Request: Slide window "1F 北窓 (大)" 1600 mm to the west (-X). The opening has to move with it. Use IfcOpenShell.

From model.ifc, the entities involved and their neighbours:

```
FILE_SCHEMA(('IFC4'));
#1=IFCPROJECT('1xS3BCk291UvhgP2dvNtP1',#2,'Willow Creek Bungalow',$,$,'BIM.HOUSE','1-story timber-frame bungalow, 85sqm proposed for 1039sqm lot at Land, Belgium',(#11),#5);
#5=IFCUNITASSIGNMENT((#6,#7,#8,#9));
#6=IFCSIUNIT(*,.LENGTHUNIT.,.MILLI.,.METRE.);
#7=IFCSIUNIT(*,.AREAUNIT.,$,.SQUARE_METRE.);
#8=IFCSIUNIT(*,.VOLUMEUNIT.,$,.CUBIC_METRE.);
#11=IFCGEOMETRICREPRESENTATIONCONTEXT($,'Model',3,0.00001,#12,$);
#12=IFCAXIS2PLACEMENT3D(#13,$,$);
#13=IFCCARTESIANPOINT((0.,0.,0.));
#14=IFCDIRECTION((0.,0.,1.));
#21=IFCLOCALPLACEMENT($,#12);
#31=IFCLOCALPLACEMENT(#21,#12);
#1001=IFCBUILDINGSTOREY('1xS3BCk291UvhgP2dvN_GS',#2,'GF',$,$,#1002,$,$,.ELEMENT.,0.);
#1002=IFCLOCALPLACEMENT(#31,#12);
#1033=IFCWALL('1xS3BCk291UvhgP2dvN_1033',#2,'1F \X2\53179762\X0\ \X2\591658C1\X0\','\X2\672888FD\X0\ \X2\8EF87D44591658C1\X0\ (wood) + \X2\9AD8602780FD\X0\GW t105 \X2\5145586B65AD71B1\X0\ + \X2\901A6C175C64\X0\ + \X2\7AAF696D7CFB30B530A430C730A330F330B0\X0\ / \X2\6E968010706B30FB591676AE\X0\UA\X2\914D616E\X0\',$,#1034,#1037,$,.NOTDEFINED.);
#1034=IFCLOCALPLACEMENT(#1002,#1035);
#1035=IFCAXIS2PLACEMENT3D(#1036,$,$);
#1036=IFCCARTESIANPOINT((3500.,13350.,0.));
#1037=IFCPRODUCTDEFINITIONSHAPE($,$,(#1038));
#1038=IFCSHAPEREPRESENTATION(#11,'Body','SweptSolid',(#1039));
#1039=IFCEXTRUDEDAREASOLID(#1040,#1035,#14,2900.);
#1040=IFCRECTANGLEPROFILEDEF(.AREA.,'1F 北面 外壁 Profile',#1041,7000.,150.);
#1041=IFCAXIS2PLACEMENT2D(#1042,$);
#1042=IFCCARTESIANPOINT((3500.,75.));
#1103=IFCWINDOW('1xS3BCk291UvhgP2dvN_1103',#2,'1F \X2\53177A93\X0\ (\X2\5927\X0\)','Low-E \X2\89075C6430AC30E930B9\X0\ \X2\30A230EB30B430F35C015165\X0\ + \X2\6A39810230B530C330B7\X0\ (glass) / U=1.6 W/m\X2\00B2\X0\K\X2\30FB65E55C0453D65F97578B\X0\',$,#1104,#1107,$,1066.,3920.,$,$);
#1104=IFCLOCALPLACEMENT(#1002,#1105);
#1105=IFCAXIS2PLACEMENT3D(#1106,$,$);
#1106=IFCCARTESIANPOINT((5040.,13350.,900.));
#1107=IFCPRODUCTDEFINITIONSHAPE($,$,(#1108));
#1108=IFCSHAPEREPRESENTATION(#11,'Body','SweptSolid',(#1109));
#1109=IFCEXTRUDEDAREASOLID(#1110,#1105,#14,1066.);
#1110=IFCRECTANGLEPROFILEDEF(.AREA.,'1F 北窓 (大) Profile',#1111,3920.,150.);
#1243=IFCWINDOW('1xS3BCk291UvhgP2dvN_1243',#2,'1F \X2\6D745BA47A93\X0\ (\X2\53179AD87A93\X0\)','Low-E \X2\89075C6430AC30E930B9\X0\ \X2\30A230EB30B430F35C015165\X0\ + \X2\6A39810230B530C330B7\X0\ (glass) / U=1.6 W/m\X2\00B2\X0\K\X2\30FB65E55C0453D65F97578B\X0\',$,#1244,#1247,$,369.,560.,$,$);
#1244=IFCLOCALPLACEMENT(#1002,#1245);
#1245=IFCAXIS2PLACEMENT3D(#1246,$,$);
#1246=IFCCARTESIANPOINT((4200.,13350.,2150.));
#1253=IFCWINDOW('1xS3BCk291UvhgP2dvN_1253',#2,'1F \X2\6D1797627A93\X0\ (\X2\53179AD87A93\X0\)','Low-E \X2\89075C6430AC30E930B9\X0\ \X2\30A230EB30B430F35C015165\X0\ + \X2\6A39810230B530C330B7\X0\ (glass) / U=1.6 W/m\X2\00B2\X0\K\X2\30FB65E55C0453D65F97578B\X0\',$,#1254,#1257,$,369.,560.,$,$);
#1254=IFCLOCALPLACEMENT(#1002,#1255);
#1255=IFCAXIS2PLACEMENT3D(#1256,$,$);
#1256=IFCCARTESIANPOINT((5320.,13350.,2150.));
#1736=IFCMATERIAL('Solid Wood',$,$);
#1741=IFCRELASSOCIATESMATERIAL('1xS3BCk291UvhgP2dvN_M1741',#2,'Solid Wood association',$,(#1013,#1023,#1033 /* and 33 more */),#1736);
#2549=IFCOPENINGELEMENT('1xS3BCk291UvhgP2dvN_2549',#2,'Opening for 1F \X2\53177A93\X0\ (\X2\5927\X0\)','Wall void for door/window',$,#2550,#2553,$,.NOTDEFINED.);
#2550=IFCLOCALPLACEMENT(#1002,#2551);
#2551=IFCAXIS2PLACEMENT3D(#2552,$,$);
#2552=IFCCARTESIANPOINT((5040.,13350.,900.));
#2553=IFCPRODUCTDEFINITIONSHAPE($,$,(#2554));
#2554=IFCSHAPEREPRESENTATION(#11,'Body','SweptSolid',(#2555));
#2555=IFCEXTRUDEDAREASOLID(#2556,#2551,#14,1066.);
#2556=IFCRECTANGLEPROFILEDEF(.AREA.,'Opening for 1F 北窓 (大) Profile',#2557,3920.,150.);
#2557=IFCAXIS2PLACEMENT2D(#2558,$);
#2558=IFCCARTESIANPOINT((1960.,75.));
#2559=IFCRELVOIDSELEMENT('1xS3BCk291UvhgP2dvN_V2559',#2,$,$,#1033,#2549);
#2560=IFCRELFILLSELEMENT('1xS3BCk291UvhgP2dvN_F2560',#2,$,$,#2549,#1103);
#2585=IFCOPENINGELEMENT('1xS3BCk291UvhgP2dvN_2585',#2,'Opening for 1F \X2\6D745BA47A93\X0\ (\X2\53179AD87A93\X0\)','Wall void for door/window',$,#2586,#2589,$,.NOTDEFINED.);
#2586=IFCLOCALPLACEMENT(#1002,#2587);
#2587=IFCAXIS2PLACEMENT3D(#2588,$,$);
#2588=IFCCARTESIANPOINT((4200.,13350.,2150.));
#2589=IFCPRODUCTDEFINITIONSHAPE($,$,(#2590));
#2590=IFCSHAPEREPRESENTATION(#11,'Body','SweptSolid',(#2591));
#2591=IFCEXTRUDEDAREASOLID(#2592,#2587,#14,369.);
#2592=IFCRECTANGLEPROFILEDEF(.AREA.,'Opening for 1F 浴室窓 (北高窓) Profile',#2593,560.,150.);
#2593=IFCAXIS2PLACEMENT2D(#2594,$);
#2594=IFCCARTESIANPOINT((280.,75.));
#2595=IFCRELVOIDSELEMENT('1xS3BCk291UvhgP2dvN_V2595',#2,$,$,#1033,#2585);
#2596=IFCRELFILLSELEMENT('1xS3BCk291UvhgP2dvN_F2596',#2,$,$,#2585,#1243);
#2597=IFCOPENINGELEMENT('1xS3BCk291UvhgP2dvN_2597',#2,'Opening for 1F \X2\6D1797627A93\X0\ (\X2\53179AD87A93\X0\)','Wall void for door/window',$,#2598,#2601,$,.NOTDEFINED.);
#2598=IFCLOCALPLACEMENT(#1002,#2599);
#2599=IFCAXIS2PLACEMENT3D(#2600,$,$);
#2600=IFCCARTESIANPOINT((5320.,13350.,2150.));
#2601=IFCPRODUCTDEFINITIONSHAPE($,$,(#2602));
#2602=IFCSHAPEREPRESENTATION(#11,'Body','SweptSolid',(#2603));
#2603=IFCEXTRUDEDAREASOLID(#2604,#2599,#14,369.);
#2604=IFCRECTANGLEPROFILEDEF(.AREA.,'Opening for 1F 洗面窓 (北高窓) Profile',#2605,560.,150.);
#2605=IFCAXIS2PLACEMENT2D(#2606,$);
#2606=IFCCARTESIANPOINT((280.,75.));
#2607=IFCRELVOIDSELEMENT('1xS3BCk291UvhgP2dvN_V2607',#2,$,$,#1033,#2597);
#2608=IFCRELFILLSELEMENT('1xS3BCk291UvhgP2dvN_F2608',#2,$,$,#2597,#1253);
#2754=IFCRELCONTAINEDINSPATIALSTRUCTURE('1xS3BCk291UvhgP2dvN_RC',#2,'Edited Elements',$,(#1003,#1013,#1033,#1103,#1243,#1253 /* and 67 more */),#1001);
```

```python
import ifcopenshell
import ifcopenshell.api.geometry
import ifcopenshell.util.placement
import ifcopenshell.util.unit

model = ifcopenshell.open("model.ifc")
unit_scale = ifcopenshell.util.unit.calculate_unit_scale(model)

window = model.by_id(1103)
opening = window.FillsVoids[0].RelatingOpeningElement
wall = opening.VoidsElements[0].RelatingBuildingElement

wall_matrix = ifcopenshell.util.placement.get_local_placement(wall.ObjectPlacement)
shift = wall_matrix[:3, 0] * -1.6 / unit_scale
before = ifcopenshell.util.placement.get_local_placement(window.ObjectPlacement)[:3, 3].copy()

# The window is not placed relative to its opening, so move both.
for product in (opening, window):
    matrix = ifcopenshell.util.placement.get_local_placement(product.ObjectPlacement)
    matrix[:3, 3] += shift
    ifcopenshell.api.geometry.edit_object_placement(model, product=product, matrix=matrix, is_si=False)

after = ifcopenshell.util.placement.get_local_placement(window.ObjectPlacement)[:3, 3]
print("window moved by", (after - before).round(3) + 0.0)

model.write("model_updated.ifc")
```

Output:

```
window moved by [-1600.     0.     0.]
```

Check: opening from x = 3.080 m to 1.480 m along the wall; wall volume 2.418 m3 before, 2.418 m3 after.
